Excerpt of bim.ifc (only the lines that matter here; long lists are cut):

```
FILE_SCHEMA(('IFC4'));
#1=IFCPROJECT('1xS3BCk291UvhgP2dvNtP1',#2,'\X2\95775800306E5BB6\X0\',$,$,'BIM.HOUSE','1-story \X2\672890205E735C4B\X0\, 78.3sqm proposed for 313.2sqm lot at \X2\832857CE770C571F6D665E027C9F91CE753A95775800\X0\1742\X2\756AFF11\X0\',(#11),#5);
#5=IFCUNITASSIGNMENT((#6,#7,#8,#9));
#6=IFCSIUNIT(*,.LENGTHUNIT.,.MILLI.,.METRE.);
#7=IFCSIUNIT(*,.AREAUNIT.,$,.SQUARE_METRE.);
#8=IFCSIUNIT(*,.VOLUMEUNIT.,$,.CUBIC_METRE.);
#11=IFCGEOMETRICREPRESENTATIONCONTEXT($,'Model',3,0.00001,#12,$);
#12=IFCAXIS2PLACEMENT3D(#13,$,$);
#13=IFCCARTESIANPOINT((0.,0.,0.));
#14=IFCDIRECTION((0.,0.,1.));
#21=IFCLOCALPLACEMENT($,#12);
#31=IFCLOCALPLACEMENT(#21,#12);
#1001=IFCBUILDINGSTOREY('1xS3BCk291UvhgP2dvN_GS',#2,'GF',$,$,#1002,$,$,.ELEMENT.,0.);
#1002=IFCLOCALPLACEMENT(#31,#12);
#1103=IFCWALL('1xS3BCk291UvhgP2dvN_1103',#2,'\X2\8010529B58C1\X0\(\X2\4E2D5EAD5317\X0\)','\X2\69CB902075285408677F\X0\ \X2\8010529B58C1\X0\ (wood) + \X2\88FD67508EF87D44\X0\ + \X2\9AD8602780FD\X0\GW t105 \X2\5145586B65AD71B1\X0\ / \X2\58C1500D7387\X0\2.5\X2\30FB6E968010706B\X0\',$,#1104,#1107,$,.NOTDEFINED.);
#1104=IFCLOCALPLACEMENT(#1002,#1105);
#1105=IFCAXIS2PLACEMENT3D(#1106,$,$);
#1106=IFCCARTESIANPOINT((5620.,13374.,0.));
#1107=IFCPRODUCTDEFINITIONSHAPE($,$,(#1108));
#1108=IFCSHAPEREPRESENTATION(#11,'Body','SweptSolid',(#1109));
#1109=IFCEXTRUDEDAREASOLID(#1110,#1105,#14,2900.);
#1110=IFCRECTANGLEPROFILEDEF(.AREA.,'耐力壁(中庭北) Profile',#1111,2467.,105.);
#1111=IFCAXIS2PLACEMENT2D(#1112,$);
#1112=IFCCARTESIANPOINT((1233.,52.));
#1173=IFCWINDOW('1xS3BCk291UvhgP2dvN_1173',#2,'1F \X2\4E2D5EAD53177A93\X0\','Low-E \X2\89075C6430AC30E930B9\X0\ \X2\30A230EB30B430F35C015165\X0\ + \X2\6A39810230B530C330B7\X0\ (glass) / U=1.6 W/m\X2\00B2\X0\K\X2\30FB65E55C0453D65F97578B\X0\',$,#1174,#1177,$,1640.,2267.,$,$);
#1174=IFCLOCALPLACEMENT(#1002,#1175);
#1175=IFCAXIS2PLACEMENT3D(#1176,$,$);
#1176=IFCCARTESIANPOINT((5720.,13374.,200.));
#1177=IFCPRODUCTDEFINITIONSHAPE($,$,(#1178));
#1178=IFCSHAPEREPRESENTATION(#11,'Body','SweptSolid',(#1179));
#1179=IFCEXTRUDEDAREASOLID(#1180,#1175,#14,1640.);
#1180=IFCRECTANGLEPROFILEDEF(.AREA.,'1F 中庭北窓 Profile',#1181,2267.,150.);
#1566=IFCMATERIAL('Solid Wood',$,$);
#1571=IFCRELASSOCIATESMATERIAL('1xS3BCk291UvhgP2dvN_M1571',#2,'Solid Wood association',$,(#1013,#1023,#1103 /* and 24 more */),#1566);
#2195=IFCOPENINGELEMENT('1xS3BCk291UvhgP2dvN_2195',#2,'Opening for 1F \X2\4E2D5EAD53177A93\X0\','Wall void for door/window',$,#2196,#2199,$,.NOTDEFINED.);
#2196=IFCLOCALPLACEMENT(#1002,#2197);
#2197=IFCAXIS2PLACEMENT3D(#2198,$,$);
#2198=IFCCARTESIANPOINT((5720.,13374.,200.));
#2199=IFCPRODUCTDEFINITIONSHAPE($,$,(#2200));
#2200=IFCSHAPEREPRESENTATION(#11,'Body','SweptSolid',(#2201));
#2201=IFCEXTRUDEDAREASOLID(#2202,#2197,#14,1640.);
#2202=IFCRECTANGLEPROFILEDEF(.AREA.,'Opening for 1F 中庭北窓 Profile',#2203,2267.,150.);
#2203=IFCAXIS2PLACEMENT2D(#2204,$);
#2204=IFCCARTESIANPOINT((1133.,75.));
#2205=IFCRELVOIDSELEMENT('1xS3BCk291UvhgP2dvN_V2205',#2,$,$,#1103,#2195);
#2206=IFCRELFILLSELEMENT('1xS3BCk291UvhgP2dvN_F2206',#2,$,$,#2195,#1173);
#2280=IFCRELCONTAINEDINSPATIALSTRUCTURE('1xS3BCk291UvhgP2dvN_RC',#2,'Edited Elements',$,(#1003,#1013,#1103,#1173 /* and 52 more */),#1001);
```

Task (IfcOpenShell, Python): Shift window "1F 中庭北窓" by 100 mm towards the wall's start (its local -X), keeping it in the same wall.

```python
import ifcopenshell
import ifcopenshell.api.geometry
import ifcopenshell.util.placement

model = ifcopenshell.open("bim.ifc")

window = model.by_guid("1xS3BCk291UvhgP2dvN_1173")
opening = window.FillsVoids[0].RelatingOpeningElement
wall = opening.VoidsElements[0].RelatingBuildingElement

wall_matrix = ifcopenshell.util.placement.get_local_placement(wall.ObjectPlacement)
shift = wall_matrix[:3, 0] * -100.0
before = ifcopenshell.util.placement.get_local_placement(window.ObjectPlacement)[:3, 3].copy()

# The window is not placed relative to its opening, so move both.
for product in (opening, window):
    matrix = ifcopenshell.util.placement.get_local_placement(product.ObjectPlacement)
    matrix[:3, 3] += shift
    ifcopenshell.api.geometry.edit_object_placement(model, product=product, matrix=matrix, is_si=False)

after = ifcopenshell.util.placement.get_local_placement(window.ObjectPlacement)[:3, 3]
print("window moved by", (after - before).round(3) + 0.0)

model.write("bim_rev.ifc")
```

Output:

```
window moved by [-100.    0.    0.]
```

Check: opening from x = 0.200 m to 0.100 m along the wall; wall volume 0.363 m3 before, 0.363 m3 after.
